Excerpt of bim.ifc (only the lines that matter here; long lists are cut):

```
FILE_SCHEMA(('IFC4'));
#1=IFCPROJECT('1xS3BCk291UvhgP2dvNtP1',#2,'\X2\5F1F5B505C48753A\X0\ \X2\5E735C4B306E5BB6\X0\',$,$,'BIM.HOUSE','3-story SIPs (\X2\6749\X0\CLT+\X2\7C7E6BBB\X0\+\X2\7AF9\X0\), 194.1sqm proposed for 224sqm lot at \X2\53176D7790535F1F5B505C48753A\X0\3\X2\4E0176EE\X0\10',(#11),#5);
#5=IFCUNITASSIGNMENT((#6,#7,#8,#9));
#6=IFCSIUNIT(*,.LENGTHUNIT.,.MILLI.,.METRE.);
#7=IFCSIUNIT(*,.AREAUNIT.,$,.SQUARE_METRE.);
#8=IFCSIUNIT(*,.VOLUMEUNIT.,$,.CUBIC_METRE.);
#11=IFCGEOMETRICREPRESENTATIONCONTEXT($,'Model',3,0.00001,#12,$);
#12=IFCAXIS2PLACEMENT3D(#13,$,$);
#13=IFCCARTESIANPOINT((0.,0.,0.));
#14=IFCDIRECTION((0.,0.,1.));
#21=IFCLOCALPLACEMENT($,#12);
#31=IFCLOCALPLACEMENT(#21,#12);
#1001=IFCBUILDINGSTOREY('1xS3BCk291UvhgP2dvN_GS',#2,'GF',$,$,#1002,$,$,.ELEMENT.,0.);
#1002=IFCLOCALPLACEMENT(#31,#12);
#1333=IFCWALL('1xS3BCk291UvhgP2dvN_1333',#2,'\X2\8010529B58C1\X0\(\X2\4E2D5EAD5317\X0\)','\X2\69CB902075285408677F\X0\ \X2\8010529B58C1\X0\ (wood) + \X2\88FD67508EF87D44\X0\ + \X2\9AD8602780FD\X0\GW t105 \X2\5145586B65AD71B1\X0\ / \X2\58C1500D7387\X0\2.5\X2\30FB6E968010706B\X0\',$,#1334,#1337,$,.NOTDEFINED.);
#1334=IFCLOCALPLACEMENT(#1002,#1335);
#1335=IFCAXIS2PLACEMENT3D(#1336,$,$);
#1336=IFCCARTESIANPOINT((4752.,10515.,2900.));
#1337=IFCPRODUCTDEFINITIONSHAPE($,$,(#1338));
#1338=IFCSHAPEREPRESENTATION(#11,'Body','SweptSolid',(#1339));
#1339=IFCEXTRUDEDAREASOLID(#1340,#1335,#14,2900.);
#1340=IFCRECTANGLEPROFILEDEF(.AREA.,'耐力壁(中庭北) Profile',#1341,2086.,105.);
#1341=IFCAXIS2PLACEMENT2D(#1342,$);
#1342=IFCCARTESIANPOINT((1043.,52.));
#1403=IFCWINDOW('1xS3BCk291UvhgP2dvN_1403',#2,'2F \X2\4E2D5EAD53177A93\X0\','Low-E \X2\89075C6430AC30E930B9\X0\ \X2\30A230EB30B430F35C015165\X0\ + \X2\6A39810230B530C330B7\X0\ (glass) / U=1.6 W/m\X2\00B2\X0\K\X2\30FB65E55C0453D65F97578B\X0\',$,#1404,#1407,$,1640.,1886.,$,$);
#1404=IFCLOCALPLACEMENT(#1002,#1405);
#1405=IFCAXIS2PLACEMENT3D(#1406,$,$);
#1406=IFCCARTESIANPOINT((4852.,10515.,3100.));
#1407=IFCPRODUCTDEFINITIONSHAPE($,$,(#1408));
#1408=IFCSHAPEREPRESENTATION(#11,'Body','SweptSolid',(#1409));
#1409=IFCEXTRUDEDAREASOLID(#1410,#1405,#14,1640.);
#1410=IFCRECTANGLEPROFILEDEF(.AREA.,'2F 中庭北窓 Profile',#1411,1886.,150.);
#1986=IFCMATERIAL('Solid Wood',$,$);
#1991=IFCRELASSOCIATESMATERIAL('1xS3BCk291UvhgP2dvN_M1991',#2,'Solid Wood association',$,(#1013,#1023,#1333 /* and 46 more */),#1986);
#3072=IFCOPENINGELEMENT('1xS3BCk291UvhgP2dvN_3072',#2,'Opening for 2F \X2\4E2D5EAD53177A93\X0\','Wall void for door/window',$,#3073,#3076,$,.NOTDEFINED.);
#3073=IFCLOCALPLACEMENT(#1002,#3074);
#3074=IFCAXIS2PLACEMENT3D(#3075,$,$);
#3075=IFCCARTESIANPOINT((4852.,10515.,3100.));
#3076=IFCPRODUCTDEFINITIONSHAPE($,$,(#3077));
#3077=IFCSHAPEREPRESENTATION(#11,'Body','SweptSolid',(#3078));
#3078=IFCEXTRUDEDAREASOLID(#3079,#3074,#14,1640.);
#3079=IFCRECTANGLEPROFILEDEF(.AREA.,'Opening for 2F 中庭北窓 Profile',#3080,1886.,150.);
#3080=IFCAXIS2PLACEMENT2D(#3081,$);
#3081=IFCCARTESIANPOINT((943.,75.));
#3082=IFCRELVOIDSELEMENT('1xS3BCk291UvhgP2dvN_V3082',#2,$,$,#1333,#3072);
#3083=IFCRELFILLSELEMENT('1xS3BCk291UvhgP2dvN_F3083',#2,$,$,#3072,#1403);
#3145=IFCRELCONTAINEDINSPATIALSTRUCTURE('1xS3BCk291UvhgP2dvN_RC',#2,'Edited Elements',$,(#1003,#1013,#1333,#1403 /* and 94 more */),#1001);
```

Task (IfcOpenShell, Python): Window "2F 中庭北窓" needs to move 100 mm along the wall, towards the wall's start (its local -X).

```python
import ifcopenshell
import ifcopenshell.api.geometry
import ifcopenshell.util.placement
import ifcopenshell.util.unit

model = ifcopenshell.open("bim.ifc")
unit_scale = ifcopenshell.util.unit.calculate_unit_scale(model)

window = model.by_guid("1xS3BCk291UvhgP2dvN_1403")
opening = window.FillsVoids[0].RelatingOpeningElement
wall = opening.VoidsElements[0].RelatingBuildingElement

wall_matrix = ifcopenshell.util.placement.get_local_placement(wall.ObjectPlacement)
shift = wall_matrix[:3, 0] * -0.1 / unit_scale
before = ifcopenshell.util.placement.get_local_placement(window.ObjectPlacement)[:3, 3].copy()

# The window is not placed relative to its opening, so move both.
for product in (opening, window):
    matrix = ifcopenshell.util.placement.get_local_placement(product.ObjectPlacement)
    matrix[:3, 3] += shift
    ifcopenshell.api.geometry.edit_object_placement(model, product=product, matrix=matrix, is_si=False)

after = ifcopenshell.util.placement.get_local_placement(window.ObjectPlacement)[:3, 3]
print("window moved by", (after - before).round(3) + 0.0)

model.write("bim_edited.ifc")
```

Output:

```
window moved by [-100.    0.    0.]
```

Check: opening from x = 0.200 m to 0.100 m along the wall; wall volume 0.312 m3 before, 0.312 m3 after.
